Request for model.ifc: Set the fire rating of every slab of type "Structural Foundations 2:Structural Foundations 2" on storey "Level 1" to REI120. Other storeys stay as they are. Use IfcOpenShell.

First a look at what the model holds.

```python
import ifcopenshell
import ifcopenshell.util.element

model = ifcopenshell.open("model.ifc")
print(model.schema)
storey = next(s for s in model.by_type("IfcBuildingStorey") if s.Name == "Level 1")
slabs = [e for e in ifcopenshell.util.element.get_decomposition(storey) if e.is_a("IfcSlab")]
seen = {}
for e in slabs:
    element_type = ifcopenshell.util.element.get_type(e)
    key = (element_type.Name if element_type != e and element_type else None, ifcopenshell.util.element.get_pset(e, "Pset_SlabCommon", "FireRating"))
    seen[key] = seen.get(key, 0) + 1
for (name, value), count in sorted(seen.items(), key=str):
    print(count, "x", name, "|", value)
```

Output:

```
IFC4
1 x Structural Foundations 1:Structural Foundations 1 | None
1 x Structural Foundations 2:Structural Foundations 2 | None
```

```python
import ifcopenshell
import ifcopenshell.api.pset
import ifcopenshell.util.element

model = ifcopenshell.open("model.ifc")

storey = next(s for s in model.by_type("IfcBuildingStorey") if s.Name == "Level 1")
slabs = [e for e in ifcopenshell.util.element.get_decomposition(storey) if e.is_a("IfcSlab")]

count = 0
for e in slabs:
    element_type = ifcopenshell.util.element.get_type(e)
    if element_type in (None, e) or element_type.Name != "Structural Foundations 2:Structural Foundations 2":
        continue
    # add_pset returns the element's existing set when there is one.
    pset = ifcopenshell.api.pset.add_pset(model, product=e, name="Pset_SlabCommon")
    ifcopenshell.api.pset.edit_pset(model, pset=pset, properties={"FireRating": "REI120"})
    count += 1

print(count, "slabs updated")

model.write("model_v2.ifc")
```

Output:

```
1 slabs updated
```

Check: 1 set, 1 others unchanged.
